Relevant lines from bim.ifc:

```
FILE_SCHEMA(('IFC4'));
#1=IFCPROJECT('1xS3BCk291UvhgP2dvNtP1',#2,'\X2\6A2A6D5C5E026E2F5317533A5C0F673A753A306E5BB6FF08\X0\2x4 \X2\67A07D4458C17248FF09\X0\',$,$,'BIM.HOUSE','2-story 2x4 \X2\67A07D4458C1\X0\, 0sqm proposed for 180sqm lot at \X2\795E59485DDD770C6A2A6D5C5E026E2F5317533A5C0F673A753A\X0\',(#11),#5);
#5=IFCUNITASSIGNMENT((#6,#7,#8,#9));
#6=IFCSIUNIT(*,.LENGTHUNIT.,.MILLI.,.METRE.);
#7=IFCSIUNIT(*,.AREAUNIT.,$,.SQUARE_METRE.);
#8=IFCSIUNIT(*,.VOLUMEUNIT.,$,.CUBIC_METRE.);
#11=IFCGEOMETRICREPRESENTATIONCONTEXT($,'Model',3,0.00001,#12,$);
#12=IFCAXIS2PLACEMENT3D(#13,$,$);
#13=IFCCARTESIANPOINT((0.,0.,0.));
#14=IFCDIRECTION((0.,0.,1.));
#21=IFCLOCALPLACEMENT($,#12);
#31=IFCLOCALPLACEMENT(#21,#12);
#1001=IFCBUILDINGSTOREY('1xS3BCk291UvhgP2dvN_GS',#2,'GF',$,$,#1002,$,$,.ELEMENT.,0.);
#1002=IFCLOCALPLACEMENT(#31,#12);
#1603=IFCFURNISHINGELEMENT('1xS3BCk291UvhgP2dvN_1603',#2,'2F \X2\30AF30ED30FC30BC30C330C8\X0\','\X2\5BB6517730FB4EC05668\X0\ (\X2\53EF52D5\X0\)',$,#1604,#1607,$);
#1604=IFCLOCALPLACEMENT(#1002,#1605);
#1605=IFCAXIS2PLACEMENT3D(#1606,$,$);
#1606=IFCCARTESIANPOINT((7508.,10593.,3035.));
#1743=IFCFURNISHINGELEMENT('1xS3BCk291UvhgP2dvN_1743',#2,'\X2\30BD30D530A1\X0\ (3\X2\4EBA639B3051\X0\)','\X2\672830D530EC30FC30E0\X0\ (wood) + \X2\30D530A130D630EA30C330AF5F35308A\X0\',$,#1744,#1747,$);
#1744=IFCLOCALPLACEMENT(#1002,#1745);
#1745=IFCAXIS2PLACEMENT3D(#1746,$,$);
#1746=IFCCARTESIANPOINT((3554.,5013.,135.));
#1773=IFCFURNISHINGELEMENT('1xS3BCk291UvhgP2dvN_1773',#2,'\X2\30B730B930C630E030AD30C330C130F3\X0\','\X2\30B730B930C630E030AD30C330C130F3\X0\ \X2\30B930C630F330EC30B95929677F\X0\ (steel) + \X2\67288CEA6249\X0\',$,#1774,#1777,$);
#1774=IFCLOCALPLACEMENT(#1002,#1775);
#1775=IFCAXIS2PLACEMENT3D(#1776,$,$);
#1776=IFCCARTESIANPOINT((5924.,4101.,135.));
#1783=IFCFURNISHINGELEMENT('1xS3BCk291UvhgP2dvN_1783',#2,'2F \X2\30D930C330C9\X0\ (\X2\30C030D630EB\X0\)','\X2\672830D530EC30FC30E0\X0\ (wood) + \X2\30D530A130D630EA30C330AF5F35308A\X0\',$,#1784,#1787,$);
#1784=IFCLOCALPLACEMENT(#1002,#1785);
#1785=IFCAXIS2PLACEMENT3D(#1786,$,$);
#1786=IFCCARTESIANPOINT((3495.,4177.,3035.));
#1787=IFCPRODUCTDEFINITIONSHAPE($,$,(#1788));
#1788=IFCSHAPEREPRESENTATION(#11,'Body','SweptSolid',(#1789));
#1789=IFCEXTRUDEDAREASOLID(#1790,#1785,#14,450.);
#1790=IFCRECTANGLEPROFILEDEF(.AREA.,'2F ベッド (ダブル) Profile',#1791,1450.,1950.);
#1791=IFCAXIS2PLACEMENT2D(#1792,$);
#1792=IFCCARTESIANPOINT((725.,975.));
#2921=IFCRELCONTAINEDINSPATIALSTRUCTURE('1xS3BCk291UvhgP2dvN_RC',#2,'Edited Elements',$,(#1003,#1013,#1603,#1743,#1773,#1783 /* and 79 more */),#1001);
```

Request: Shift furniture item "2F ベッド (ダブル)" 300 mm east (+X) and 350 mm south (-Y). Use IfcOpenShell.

```python
import ifcopenshell
import ifcopenshell.api.geometry
import ifcopenshell.util.placement
import ifcopenshell.util.unit

model = ifcopenshell.open("bim.ifc")
unit_scale = ifcopenshell.util.unit.calculate_unit_scale(model)

item = model.by_id(1783)
matrix = ifcopenshell.util.placement.get_local_placement(item.ObjectPlacement)
matrix[0, 3] += 0.3 / unit_scale
matrix[1, 3] -= 0.35 / unit_scale
ifcopenshell.api.geometry.edit_object_placement(model, product=item, matrix=matrix, is_si=False)

print(ifcopenshell.util.placement.get_local_placement(item.ObjectPlacement).round(3) + 0.0)

model.write("bim_edited.ifc")
```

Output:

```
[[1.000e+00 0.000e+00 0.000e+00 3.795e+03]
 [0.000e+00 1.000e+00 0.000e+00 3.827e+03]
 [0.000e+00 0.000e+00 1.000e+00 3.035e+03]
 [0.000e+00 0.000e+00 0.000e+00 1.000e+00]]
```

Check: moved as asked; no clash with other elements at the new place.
